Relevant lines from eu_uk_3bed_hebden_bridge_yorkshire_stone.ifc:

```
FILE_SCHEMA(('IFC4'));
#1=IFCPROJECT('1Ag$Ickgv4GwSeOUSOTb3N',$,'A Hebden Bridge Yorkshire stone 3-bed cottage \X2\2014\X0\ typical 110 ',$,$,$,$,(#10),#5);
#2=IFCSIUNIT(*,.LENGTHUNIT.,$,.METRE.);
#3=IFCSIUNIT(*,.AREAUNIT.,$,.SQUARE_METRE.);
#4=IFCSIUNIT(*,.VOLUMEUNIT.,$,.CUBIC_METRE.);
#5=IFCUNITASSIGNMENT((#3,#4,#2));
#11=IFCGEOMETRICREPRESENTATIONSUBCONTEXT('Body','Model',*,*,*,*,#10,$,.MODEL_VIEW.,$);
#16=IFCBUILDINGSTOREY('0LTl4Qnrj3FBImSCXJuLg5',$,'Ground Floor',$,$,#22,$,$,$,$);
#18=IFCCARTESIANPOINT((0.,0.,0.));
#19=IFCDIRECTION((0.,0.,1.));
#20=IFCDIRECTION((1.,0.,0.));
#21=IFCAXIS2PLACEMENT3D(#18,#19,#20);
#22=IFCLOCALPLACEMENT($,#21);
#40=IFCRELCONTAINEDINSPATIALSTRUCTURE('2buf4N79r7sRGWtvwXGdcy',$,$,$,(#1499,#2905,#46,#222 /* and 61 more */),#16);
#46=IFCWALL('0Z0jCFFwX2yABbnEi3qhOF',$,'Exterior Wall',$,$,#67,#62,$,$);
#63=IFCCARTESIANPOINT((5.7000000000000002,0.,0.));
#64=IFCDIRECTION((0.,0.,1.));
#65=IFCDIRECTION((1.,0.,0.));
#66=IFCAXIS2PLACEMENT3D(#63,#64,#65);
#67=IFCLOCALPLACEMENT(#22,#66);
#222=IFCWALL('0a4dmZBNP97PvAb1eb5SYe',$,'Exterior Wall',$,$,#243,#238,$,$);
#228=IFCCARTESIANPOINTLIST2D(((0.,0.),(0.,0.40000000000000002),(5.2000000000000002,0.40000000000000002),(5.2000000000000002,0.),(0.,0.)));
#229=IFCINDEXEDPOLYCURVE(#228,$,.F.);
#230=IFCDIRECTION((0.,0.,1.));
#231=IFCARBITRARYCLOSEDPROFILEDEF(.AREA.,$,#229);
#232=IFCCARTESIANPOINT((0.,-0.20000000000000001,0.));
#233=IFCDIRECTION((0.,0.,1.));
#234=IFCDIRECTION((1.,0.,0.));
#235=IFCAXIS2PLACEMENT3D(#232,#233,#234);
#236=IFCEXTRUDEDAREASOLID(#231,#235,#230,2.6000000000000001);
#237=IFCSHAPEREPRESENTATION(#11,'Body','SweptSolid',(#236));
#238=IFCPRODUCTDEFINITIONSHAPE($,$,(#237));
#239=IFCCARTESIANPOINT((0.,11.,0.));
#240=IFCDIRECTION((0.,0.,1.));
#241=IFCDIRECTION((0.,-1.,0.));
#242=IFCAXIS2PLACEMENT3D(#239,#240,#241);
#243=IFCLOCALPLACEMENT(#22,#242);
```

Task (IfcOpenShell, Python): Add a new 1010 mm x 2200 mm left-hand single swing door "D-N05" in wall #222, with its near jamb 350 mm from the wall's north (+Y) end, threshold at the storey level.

```python
import numpy as np
import ifcopenshell
import ifcopenshell.api.feature
import ifcopenshell.api.geometry
import ifcopenshell.api.root
import ifcopenshell.api.spatial
import ifcopenshell.geom
import ifcopenshell.util.element
import ifcopenshell.util.placement
import ifcopenshell.util.representation
import ifcopenshell.util.shape
import ifcopenshell.util.unit

model = ifcopenshell.open("eu_uk_3bed_hebden_bridge_yorkshire_stone.ifc")
unit_scale = ifcopenshell.util.unit.calculate_unit_scale(model)
settings = ifcopenshell.geom.settings()


def volume(element):
    """Net volume in cubic metres, openings subtracted."""
    shape = ifcopenshell.geom.create_shape(settings, element)
    return ifcopenshell.util.shape.get_volume(shape.geometry)


wall = model.by_guid("0a4dmZBNP97PvAb1eb5SYe")
storey = ifcopenshell.util.element.get_container(wall, ifc_class="IfcBuildingStorey")
context = ifcopenshell.util.representation.get_context(model, "Model", "Body", "MODEL_VIEW")
before = volume(wall)

width, height, from_end, sill = 1.01, 2.2, 0.35, 0.0  # metres

# The wall runs along its own X axis, and the end named is its -X end.
wall_shape = ifcopenshell.geom.create_shape(settings, wall)
x, y, z = ifcopenshell.util.shape.get_vertices(wall_shape.geometry).T
start = x.min() + from_end
face, thickness = float(y.min()), float(y.max() - y.min())
wall_matrix = ifcopenshell.util.placement.get_local_placement(wall.ObjectPlacement)
level = ifcopenshell.util.placement.get_local_placement(storey.ObjectPlacement)[2, 3]


def in_wall(x, y):
    """Placement at x, y metres in the wall's axes, at sill height."""
    matrix = wall_matrix.copy()
    matrix[:, 3] = wall_matrix @ np.array([x / unit_scale, y / unit_scale, 0.0, 1.0])
    matrix[2, 3] = level + sill / unit_scale
    return matrix


# Opening: a box that overshoots both wall faces by 50 mm.
opening = ifcopenshell.api.root.create_entity(model, ifc_class="IfcOpeningElement", predefined_type="OPENING")
box = ifcopenshell.api.geometry.add_wall_representation(
    model, context=context, length=width, height=height, thickness=thickness + 0.1
)
ifcopenshell.api.geometry.assign_representation(model, product=opening, representation=box)
ifcopenshell.api.geometry.edit_object_placement(model, product=opening, matrix=in_wall(start, face - 0.05), is_si=False)
ifcopenshell.api.feature.add_feature(model, feature=opening, element=wall)

door = ifcopenshell.api.root.create_entity(model, ifc_class="IfcDoor", name="D-N05", predefined_type="DOOR")
door.OverallWidth, door.OverallHeight = width / unit_scale, height / unit_scale
door.OperationType = "SINGLE_SWING_LEFT"
body = ifcopenshell.api.geometry.add_door_representation(
    model,
    context=context,
    overall_width=door.OverallWidth,
    overall_height=door.OverallHeight,
    operation_type="SINGLE_SWING_LEFT",
    lining_properties={"LiningDepth": thickness / unit_scale, "ThresholdDepth": thickness / unit_scale},
)
ifcopenshell.api.geometry.assign_representation(model, product=door, representation=body)
ifcopenshell.api.spatial.assign_container(model, products=[door], relating_structure=storey)
ifcopenshell.api.feature.add_filling(model, opening=opening, element=door)

# The lining spans the wall, so the door starts at the wall face.
ifcopenshell.api.geometry.edit_object_placement(model, product=door, matrix=in_wall(start, face), is_si=False)

after = volume(wall)

print(f"wall volume {before:.3f} -> {after:.3f} m3")

model.write("eu_uk_3bed_hebden_bridge_yorkshire_stone_edited.ifc")
```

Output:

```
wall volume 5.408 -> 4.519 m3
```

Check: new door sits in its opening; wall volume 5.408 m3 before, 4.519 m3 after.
